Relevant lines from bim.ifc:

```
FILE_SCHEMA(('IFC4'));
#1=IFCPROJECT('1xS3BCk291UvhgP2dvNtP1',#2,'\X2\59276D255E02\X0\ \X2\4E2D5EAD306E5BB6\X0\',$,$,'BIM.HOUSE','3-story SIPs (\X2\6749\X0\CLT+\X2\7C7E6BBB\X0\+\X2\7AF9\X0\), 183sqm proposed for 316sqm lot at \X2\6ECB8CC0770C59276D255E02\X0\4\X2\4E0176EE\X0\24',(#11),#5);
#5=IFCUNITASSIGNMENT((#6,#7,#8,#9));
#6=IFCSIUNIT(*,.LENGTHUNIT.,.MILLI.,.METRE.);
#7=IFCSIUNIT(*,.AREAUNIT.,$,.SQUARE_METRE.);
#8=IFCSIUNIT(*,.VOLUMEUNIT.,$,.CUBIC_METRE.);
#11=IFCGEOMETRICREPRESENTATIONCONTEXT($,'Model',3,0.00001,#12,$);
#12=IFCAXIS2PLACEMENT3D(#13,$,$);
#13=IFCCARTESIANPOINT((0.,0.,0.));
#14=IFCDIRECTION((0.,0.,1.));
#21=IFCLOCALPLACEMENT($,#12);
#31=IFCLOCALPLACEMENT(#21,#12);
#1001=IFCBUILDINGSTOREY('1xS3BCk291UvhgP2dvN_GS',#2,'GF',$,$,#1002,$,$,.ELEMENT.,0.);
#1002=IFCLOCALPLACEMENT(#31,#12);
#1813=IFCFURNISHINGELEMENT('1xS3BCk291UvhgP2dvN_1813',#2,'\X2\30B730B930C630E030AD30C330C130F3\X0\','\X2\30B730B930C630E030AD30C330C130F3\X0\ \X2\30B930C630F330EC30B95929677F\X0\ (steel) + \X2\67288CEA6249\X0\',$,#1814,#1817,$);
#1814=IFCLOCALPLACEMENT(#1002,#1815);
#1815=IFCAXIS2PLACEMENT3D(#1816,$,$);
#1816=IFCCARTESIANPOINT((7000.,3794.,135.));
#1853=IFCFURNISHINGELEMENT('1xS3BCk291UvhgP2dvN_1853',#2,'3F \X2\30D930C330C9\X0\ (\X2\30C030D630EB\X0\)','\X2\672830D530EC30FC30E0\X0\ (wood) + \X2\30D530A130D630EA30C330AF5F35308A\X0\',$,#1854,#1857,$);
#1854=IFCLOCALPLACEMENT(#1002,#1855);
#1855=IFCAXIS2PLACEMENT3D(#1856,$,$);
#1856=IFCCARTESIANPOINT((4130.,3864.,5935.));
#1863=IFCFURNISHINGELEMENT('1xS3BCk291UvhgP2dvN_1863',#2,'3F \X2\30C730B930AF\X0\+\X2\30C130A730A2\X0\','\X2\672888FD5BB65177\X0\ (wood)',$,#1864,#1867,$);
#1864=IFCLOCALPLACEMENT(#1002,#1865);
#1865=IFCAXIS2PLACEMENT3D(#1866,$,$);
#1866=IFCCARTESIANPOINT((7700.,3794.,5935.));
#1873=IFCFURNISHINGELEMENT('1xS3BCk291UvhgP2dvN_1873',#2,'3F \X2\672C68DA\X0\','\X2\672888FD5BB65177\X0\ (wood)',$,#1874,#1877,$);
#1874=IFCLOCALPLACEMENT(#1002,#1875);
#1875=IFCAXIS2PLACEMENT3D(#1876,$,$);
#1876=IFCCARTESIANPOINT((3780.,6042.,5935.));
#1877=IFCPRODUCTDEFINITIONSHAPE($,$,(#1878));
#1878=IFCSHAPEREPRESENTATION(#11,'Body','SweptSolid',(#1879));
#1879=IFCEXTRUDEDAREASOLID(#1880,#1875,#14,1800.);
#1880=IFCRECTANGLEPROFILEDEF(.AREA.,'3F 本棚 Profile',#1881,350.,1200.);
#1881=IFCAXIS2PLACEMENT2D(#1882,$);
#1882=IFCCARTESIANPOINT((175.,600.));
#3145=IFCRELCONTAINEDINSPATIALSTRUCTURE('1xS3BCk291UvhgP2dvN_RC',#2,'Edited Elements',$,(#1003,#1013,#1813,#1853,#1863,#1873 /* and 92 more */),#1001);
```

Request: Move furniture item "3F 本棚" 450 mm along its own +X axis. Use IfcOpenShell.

```python
import ifcopenshell
import ifcopenshell.api.geometry
import ifcopenshell.util.placement

model = ifcopenshell.open("bim.ifc")

item = model.by_id(1873)
matrix = ifcopenshell.util.placement.get_local_placement(item.ObjectPlacement)
matrix[:3, 3] += matrix[:3, 0] * 450.0
ifcopenshell.api.geometry.edit_object_placement(model, product=item, matrix=matrix, is_si=False)

print(ifcopenshell.util.placement.get_local_placement(item.ObjectPlacement).round(3) + 0.0)

model.write("bim-out.ifc")
```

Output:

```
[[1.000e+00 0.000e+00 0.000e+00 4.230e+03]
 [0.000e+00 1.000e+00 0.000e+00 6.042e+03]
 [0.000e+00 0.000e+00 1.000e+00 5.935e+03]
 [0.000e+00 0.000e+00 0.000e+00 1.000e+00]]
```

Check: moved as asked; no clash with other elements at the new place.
